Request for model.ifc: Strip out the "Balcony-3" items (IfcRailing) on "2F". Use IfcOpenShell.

First a look at what the model holds.

```python
import ifcopenshell
import ifcopenshell.util.element

model = ifcopenshell.open("model.ifc")
print(model.schema)
storey = next(s for s in model.by_type("IfcBuildingStorey") if s.Name == "2F")
railings = [e for e in ifcopenshell.util.element.get_decomposition(storey) if e.is_a("IfcRailing")]
seen = {}
for e in railings:
    element_type = ifcopenshell.util.element.get_type(e)
    name = element_type.Name if element_type not in (None, e) else None
    seen[name] = seen.get(name, 0) + 1
for name, count in sorted(seen.items(), key=str):
    print(count, "x", name)
```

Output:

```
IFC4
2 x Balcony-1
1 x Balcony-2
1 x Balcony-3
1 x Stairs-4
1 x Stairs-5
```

```python
import ifcopenshell
import ifcopenshell.api.root
import ifcopenshell.util.element

model = ifcopenshell.open("model.ifc")

storey = next(s for s in model.by_type("IfcBuildingStorey") if s.Name == "2F")
railings = [e for e in ifcopenshell.util.element.get_decomposition(storey) if e.is_a("IfcRailing")]
targets = [e for e in railings if (t := ifcopenshell.util.element.get_type(e)) not in (None, e) and t.Name == "Balcony-3"]

for e in targets:
    ifcopenshell.api.root.remove_product(model, product=e)
print(len(targets), "removed")

model.write("model_edited.ifc")
```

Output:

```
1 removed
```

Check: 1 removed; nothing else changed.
